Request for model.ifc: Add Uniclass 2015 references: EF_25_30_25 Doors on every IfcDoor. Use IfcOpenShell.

First a look at what the model holds.

```python
import ifcopenshell

model = ifcopenshell.open("model.ifc")
print(model.schema)
print("classifications:", [c.Name for c in model.by_type("IfcClassification")])
for ifc_class in ("IfcDoor", "IfcRoof", "IfcStair", "IfcWall", "IfcWindow"):
    print(ifc_class, len(model.by_type(ifc_class)))
```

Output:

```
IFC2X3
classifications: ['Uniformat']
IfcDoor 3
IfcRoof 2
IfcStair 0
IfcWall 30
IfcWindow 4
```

```python
import ifcopenshell
import ifcopenshell.api.classification

model = ifcopenshell.open("model.ifc")

# IFC2X3 requires Source and Edition and has no link from the project to the system.
system = model.create_entity("IfcClassification", Source="NBS", Edition="2015", Name="Uniclass 2015")

codes = {
    "IfcDoor": ("EF_25_30_25", "Doors"),
}
for ifc_class, (code, name) in codes.items():
    products = model.by_type(ifc_class)
    ifcopenshell.api.classification.add_reference(
        model, products=products, classification=system, identification=code, name=name
    )
    print(code, len(products))

model.write("model_updated.ifc")
```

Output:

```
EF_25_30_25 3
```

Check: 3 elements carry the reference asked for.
